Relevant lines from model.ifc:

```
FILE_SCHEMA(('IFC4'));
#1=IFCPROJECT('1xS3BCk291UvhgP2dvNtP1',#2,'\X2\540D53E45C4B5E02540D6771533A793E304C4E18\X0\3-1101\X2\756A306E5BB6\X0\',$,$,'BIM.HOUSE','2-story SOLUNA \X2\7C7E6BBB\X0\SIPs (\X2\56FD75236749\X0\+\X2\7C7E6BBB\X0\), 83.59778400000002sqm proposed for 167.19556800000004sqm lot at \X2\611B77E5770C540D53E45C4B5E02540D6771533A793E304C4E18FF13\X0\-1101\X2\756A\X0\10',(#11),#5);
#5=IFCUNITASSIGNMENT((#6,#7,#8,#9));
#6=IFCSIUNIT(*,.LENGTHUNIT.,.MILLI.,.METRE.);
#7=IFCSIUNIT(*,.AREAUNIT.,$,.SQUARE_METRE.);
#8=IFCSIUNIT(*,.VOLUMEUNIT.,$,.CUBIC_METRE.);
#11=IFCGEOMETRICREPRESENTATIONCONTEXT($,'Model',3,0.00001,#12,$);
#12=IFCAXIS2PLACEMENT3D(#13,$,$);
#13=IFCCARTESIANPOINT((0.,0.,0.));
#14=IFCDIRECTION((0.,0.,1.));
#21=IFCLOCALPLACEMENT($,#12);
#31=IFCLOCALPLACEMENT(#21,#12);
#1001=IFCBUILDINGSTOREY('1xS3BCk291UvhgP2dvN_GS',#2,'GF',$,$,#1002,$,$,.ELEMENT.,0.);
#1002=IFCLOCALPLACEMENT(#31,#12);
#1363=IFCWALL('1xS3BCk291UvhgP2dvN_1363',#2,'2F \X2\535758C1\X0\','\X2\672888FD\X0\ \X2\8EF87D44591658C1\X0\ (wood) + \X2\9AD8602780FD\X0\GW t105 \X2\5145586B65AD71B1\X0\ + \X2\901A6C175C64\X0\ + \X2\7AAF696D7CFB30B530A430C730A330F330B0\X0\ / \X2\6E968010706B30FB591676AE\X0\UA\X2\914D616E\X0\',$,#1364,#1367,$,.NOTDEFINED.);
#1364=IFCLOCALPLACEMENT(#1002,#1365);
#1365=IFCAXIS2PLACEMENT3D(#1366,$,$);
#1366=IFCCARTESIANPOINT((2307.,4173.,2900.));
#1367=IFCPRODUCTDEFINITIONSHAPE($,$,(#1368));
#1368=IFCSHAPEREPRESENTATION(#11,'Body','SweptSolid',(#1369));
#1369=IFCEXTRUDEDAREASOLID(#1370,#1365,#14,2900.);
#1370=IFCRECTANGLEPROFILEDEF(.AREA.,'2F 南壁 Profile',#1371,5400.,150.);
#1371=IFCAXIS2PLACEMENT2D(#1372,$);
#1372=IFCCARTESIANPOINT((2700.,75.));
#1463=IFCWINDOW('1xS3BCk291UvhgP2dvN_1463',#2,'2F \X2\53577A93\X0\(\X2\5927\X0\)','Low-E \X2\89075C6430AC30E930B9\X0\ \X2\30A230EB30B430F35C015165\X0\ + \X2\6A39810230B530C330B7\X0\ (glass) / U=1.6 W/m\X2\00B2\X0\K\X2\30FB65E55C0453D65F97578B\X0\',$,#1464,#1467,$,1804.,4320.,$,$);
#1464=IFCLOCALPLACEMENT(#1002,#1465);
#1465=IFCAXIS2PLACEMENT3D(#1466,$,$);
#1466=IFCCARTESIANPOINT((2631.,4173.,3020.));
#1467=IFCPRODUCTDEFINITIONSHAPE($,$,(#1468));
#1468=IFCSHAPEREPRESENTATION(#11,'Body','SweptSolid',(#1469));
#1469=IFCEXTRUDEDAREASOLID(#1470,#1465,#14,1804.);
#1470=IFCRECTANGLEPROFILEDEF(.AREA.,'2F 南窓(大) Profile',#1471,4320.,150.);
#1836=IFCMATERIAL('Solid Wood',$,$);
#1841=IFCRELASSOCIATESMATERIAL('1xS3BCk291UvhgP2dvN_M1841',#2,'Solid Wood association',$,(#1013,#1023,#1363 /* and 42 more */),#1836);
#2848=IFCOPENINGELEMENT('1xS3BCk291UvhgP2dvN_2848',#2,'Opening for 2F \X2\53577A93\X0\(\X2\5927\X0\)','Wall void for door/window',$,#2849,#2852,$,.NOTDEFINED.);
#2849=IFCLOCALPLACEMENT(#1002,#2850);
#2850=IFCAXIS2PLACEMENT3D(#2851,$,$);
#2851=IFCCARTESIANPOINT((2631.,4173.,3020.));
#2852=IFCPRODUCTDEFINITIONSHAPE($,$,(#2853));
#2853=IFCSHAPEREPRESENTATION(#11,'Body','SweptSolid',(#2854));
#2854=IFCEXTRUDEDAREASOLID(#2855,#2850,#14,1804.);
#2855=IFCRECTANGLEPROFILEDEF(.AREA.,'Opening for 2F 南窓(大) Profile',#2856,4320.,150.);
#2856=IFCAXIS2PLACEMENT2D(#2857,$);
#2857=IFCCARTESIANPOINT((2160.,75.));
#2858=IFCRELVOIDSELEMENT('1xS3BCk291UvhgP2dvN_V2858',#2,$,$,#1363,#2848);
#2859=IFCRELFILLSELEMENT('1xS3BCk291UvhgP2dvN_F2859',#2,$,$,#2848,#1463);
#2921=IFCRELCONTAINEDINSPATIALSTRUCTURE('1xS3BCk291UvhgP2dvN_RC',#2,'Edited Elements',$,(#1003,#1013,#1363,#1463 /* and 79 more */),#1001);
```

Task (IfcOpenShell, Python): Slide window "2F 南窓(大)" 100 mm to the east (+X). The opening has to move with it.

```python
import ifcopenshell
import ifcopenshell.api.geometry
import ifcopenshell.util.placement
import ifcopenshell.util.unit

model = ifcopenshell.open("model.ifc")
unit_scale = ifcopenshell.util.unit.calculate_unit_scale(model)

window = model.by_guid("1xS3BCk291UvhgP2dvN_1463")
opening = window.FillsVoids[0].RelatingOpeningElement
wall = opening.VoidsElements[0].RelatingBuildingElement

wall_matrix = ifcopenshell.util.placement.get_local_placement(wall.ObjectPlacement)
shift = wall_matrix[:3, 0] * 0.1 / unit_scale
before = ifcopenshell.util.placement.get_local_placement(window.ObjectPlacement)[:3, 3].copy()

# The window is not placed relative to its opening, so move both.
for product in (opening, window):
    matrix = ifcopenshell.util.placement.get_local_placement(product.ObjectPlacement)
    matrix[:3, 3] += shift
    ifcopenshell.api.geometry.edit_object_placement(model, product=product, matrix=matrix, is_si=False)

after = ifcopenshell.util.placement.get_local_placement(window.ObjectPlacement)[:3, 3]
print("window moved by", (after - before).round(3) + 0.0)

model.write("model_v2.ifc")
```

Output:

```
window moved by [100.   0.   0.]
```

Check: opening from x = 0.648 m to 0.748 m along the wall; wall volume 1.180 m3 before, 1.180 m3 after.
